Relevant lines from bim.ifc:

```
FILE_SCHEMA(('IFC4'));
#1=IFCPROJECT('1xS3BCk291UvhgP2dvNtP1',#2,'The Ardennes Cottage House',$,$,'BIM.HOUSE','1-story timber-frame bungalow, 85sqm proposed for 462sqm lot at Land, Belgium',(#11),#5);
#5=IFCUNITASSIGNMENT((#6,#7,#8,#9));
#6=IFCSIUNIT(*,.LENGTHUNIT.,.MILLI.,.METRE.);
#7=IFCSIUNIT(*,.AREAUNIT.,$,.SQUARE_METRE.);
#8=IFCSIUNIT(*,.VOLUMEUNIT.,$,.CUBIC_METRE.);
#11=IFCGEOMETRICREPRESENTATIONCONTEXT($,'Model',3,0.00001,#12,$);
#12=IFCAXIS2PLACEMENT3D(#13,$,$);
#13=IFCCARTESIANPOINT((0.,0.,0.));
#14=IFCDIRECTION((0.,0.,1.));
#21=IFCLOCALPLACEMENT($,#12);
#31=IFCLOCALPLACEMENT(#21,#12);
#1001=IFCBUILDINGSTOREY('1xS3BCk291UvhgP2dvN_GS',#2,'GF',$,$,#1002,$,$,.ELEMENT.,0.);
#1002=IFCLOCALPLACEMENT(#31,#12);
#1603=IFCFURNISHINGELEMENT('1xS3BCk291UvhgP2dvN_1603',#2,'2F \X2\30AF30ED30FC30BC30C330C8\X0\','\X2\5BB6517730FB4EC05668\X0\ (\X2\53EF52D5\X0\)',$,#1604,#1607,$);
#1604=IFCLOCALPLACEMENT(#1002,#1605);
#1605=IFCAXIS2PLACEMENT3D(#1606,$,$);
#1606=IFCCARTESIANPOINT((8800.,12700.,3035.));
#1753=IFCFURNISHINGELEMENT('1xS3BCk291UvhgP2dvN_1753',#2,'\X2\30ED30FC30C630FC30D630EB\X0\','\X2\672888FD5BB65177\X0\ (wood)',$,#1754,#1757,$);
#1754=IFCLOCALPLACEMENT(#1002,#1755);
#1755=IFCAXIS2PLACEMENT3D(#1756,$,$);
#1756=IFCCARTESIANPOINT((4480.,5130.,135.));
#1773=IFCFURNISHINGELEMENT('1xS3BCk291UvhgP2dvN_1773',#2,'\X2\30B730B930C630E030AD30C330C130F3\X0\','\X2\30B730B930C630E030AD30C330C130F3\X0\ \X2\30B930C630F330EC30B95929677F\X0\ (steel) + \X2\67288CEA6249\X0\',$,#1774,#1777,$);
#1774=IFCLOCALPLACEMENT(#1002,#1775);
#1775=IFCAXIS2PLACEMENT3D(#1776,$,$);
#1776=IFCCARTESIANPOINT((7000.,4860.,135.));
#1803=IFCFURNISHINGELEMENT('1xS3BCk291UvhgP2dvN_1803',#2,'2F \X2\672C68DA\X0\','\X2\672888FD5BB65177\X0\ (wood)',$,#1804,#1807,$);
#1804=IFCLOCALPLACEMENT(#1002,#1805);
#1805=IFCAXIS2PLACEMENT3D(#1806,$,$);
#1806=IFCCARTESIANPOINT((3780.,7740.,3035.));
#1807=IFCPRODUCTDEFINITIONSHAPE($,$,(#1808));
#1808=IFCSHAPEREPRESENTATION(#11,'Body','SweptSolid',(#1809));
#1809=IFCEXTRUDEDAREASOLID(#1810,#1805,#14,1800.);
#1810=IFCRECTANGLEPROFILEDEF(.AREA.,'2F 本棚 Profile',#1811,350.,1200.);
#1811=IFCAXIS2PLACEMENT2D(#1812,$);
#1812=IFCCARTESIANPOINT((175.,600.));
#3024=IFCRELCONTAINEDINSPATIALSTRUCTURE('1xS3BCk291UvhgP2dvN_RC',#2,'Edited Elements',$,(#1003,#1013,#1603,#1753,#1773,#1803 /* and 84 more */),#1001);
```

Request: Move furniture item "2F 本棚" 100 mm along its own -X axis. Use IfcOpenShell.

```python
import ifcopenshell
import ifcopenshell.api.geometry
import ifcopenshell.util.placement
import ifcopenshell.util.unit

model = ifcopenshell.open("bim.ifc")
unit_scale = ifcopenshell.util.unit.calculate_unit_scale(model)

item = model.by_guid("1xS3BCk291UvhgP2dvN_1803")
matrix = ifcopenshell.util.placement.get_local_placement(item.ObjectPlacement)
matrix[:3, 3] -= matrix[:3, 0] * 0.1 / unit_scale
ifcopenshell.api.geometry.edit_object_placement(model, product=item, matrix=matrix, is_si=False)

print(ifcopenshell.util.placement.get_local_placement(item.ObjectPlacement).round(3) + 0.0)

model.write("bim_updated.ifc")
```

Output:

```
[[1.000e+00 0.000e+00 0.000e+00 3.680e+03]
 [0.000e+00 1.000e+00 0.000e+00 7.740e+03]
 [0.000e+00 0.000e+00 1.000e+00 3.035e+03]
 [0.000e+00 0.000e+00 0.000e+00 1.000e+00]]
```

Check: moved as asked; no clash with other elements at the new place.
